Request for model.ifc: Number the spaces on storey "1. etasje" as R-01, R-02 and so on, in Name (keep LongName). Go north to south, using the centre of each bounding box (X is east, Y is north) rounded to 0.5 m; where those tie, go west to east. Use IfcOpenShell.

First a look at what the model holds.

```python
import ifcopenshell
import ifcopenshell.util.element
import ifcopenshell.util.placement

model = ifcopenshell.open("model.ifc")
print(model.schema)
storey = next(s for s in model.by_type("IfcBuildingStorey") if s.Name == "1. etasje")
spaces = [e for e in ifcopenshell.util.element.get_decomposition(storey) if e.is_a("IfcSpace")]
for e in sorted(spaces, key=lambda e: e.id()):
    origin = ifcopenshell.util.placement.get_local_placement(e.ObjectPlacement)[:3, 3]
    print(e.id(), e.Name, e.LongName, origin.round(2) + 0.0, sep=" | ")
```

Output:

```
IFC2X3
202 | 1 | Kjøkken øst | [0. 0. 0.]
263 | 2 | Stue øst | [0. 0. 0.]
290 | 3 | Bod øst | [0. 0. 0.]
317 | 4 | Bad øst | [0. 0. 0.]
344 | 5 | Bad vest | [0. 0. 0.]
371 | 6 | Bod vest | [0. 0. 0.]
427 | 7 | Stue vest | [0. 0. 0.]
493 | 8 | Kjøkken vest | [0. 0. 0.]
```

```python
import ifcopenshell
import ifcopenshell.geom
import ifcopenshell.util.element
import ifcopenshell.util.shape

model = ifcopenshell.open("model.ifc")
settings = ifcopenshell.geom.settings()
settings.set("use-world-coords", True)


def centre(element):
    shape = ifcopenshell.geom.create_shape(settings, element)
    return ifcopenshell.util.shape.get_bbox_centroid(shape.geometry)


storey = next(s for s in model.by_type("IfcBuildingStorey") if s.Name == "1. etasje")
spaces = [e for e in ifcopenshell.util.element.get_decomposition(storey) if e.is_a("IfcSpace")]

# Insertion points can sit at a corner or the storey origin, so sort by the geometry (in metres).
centres = {e: centre(e) for e in spaces}
spaces.sort(key=lambda e: (-round(centres[e][1] / 0.5), centres[e][0]))

for i, e in enumerate(spaces, start=1):
    number = f"R-{i:02d}"
    e.Name = number
    print(e.id(), number)

model.write("model_v2.ifc")
```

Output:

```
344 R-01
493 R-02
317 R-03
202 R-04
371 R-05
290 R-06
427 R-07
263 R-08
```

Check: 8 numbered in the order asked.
